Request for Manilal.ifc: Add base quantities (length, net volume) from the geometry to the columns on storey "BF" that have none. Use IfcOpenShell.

First a look at what the model holds.

```python
import ifcopenshell
import ifcopenshell.util.element
import ifcopenshell.util.unit

model = ifcopenshell.open("Manilal.ifc")
print(model.schema)
for unit_type in ("LENGTHUNIT", "AREAUNIT", "VOLUMEUNIT"):
    print(unit_type, ifcopenshell.util.unit.calculate_unit_scale(model, unit_type))
storey = next(s for s in model.by_type("IfcBuildingStorey") if s.Name == "BF")
columns = [e for e in ifcopenshell.util.element.get_decomposition(storey) if e.is_a("IfcColumn")]
for e in sorted(columns, key=lambda e: e.id()):
    print(e.id(), e.is_a(), e.Name, list(ifcopenshell.util.element.get_psets(e, qtos_only=True)), sep=" | ")
```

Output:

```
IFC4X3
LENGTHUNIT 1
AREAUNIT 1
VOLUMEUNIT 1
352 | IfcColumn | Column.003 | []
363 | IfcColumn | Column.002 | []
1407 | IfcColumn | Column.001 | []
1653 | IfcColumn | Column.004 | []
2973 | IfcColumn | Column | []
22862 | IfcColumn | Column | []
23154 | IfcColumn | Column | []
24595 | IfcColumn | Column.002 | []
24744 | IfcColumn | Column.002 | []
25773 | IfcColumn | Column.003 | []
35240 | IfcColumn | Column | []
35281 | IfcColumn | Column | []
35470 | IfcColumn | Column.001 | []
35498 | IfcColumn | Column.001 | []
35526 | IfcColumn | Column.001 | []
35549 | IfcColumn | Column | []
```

```python
import ifcopenshell
import ifcopenshell.api.pset
import ifcopenshell.geom
import ifcopenshell.util.element
import ifcopenshell.util.shape
import ifcopenshell.util.unit

model = ifcopenshell.open("Manilal.ifc")
unit_scale = ifcopenshell.util.unit.calculate_unit_scale(model)
volume_scale = ifcopenshell.util.unit.calculate_unit_scale(model, "VOLUMEUNIT")
settings = ifcopenshell.geom.settings()

storey = next(s for s in model.by_type("IfcBuildingStorey") if s.Name == "BF")
columns = [e for e in ifcopenshell.util.element.get_decomposition(storey) if e.is_a("IfcColumn")]

for e in sorted(columns, key=lambda e: e.id()):
    if ifcopenshell.util.element.get_psets(e, qtos_only=True, should_inherit=False):
        continue
    # Geometry comes back in metres, in the element's own axes.
    shape = ifcopenshell.geom.create_shape(settings, e)
    values = {
        "Length": ifcopenshell.util.shape.get_z(shape.geometry) / unit_scale,
        "NetVolume": ifcopenshell.util.shape.get_volume(shape.geometry) / volume_scale,
    }
    qto = ifcopenshell.api.pset.add_qto(model, product=e, name="Qto_ColumnBaseQuantities")
    ifcopenshell.api.pset.edit_qto(model, qto=qto, properties=values)
    print(e.id(), {k: round(v, 3) for k, v in values.items()})

model.write("Manilal_v2.ifc")
```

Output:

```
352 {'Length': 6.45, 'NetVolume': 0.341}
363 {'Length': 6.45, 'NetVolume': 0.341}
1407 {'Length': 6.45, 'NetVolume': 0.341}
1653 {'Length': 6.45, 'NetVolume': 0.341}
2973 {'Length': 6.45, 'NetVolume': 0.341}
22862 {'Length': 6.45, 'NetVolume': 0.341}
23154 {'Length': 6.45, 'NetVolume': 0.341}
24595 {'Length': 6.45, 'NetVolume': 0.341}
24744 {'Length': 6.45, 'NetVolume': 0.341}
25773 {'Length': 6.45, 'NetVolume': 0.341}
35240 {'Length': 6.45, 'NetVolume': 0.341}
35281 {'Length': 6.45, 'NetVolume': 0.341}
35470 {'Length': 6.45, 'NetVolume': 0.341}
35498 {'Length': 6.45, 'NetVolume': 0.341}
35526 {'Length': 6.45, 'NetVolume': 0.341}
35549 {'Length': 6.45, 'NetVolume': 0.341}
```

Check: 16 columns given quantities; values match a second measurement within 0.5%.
